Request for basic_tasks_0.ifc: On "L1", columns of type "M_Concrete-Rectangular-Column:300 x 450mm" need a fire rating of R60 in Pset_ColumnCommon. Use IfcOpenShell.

First a look at what the model holds.

```python
import ifcopenshell
import ifcopenshell.util.element

model = ifcopenshell.open("basic_tasks_0.ifc")
print(model.schema)
storey = next(s for s in model.by_type("IfcBuildingStorey") if s.Name == "L1")
columns = [e for e in ifcopenshell.util.element.get_decomposition(storey) if e.is_a("IfcColumn")]
seen = {}
for e in columns:
    element_type = ifcopenshell.util.element.get_type(e)
    key = (element_type.Name if element_type != e and element_type else None, ifcopenshell.util.element.get_pset(e, "Pset_ColumnCommon", "FireRating"))
    seen[key] = seen.get(key, 0) + 1
for (name, value), count in sorted(seen.items(), key=str):
    print(count, "x", name, "|", value)
```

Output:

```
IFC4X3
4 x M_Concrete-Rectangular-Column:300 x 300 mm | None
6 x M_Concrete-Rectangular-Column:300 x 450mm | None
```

```python
import ifcopenshell
import ifcopenshell.api.pset
import ifcopenshell.util.element

model = ifcopenshell.open("basic_tasks_0.ifc")

storey = next(s for s in model.by_type("IfcBuildingStorey") if s.Name == "L1")
columns = [e for e in ifcopenshell.util.element.get_decomposition(storey) if e.is_a("IfcColumn")]

count = 0
for e in columns:
    element_type = ifcopenshell.util.element.get_type(e)
    if element_type in (None, e) or element_type.Name != "M_Concrete-Rectangular-Column:300 x 450mm":
        continue
    # add_pset returns the element's existing set when there is one.
    pset = ifcopenshell.api.pset.add_pset(model, product=e, name="Pset_ColumnCommon")
    ifcopenshell.api.pset.edit_pset(model, pset=pset, properties={"FireRating": "R60"})
    count += 1

print(count, "columns updated")

model.write("basic_tasks_0-out.ifc")
```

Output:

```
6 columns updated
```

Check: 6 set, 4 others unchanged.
